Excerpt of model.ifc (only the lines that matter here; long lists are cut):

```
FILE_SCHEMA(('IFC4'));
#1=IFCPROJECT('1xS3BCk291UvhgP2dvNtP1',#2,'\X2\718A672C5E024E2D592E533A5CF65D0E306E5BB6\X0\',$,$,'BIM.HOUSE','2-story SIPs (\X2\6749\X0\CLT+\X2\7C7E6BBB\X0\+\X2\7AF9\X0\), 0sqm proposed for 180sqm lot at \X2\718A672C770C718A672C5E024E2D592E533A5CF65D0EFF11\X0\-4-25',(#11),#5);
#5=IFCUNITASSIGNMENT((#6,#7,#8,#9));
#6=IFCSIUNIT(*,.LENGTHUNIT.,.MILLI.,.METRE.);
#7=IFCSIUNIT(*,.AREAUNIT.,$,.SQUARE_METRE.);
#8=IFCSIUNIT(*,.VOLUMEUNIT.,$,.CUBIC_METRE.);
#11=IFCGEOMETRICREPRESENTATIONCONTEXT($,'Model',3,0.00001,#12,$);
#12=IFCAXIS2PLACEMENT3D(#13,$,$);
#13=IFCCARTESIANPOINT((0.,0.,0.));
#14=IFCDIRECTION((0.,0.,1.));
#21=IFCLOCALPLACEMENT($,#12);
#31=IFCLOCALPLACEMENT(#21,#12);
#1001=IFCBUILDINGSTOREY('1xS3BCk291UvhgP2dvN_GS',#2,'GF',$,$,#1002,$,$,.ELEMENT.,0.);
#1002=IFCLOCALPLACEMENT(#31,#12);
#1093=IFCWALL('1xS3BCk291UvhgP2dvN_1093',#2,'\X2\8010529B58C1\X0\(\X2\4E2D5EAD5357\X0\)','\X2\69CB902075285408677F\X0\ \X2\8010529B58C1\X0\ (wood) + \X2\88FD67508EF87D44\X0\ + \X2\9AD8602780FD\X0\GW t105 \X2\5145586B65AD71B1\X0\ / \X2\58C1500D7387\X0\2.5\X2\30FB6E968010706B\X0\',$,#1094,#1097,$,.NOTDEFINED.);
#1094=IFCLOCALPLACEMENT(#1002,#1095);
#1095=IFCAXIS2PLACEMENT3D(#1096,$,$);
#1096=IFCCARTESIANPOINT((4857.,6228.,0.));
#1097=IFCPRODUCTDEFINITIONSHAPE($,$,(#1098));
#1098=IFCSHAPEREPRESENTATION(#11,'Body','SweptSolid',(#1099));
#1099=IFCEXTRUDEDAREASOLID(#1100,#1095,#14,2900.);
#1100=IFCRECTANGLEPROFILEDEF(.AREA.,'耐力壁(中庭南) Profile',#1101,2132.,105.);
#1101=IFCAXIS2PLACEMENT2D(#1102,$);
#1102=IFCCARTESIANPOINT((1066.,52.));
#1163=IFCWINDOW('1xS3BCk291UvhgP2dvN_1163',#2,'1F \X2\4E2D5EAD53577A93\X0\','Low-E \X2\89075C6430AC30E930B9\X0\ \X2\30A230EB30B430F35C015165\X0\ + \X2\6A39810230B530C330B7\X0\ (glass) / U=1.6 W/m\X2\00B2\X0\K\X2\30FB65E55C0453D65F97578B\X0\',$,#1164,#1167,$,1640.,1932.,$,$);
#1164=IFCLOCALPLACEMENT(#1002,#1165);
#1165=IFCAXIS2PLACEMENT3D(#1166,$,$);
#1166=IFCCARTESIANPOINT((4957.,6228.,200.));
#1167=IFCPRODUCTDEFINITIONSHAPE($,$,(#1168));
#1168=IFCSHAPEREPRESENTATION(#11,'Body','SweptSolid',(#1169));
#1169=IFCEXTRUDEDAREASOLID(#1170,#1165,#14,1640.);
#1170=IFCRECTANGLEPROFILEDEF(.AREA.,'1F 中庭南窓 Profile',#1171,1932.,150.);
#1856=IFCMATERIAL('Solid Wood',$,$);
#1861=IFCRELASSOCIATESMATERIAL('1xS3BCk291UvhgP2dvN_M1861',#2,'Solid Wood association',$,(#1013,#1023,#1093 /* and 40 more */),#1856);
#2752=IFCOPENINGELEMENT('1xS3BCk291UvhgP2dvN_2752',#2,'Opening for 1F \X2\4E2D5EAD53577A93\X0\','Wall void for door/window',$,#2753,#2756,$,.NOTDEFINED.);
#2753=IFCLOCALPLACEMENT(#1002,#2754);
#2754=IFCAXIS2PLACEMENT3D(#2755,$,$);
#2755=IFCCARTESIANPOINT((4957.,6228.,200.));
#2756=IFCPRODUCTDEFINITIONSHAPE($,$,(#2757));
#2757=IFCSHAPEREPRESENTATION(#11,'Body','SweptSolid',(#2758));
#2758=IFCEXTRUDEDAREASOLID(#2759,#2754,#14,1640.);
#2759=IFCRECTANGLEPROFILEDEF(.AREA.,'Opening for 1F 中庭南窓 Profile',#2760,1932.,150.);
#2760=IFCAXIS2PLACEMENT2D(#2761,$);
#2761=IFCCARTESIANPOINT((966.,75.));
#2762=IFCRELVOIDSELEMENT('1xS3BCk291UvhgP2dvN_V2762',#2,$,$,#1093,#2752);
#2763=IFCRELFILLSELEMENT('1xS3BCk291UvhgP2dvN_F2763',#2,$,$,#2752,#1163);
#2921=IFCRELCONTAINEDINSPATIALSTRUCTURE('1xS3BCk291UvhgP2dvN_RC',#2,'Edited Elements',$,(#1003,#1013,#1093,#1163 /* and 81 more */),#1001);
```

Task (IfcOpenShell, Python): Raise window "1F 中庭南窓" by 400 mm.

```python
import numpy as np
import ifcopenshell
import ifcopenshell.api.geometry
import ifcopenshell.util.placement
import ifcopenshell.util.unit

model = ifcopenshell.open("model.ifc")
unit_scale = ifcopenshell.util.unit.calculate_unit_scale(model)

window = model.by_guid("1xS3BCk291UvhgP2dvN_1163")
opening = window.FillsVoids[0].RelatingOpeningElement
dz = 0.4 / unit_scale

shift = np.array([0.0, 0.0, dz])
# The window is not placed relative to its opening, so move both.
for product in (opening, window):
    matrix = ifcopenshell.util.placement.get_local_placement(product.ObjectPlacement)
    matrix[:3, 3] += shift
    ifcopenshell.api.geometry.edit_object_placement(model, product=product, matrix=matrix, is_si=False)

print(f"moved by {dz * unit_scale:+.3f} m")

model.write("model_v2.ifc")
```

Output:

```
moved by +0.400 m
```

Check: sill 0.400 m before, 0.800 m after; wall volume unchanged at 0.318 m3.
